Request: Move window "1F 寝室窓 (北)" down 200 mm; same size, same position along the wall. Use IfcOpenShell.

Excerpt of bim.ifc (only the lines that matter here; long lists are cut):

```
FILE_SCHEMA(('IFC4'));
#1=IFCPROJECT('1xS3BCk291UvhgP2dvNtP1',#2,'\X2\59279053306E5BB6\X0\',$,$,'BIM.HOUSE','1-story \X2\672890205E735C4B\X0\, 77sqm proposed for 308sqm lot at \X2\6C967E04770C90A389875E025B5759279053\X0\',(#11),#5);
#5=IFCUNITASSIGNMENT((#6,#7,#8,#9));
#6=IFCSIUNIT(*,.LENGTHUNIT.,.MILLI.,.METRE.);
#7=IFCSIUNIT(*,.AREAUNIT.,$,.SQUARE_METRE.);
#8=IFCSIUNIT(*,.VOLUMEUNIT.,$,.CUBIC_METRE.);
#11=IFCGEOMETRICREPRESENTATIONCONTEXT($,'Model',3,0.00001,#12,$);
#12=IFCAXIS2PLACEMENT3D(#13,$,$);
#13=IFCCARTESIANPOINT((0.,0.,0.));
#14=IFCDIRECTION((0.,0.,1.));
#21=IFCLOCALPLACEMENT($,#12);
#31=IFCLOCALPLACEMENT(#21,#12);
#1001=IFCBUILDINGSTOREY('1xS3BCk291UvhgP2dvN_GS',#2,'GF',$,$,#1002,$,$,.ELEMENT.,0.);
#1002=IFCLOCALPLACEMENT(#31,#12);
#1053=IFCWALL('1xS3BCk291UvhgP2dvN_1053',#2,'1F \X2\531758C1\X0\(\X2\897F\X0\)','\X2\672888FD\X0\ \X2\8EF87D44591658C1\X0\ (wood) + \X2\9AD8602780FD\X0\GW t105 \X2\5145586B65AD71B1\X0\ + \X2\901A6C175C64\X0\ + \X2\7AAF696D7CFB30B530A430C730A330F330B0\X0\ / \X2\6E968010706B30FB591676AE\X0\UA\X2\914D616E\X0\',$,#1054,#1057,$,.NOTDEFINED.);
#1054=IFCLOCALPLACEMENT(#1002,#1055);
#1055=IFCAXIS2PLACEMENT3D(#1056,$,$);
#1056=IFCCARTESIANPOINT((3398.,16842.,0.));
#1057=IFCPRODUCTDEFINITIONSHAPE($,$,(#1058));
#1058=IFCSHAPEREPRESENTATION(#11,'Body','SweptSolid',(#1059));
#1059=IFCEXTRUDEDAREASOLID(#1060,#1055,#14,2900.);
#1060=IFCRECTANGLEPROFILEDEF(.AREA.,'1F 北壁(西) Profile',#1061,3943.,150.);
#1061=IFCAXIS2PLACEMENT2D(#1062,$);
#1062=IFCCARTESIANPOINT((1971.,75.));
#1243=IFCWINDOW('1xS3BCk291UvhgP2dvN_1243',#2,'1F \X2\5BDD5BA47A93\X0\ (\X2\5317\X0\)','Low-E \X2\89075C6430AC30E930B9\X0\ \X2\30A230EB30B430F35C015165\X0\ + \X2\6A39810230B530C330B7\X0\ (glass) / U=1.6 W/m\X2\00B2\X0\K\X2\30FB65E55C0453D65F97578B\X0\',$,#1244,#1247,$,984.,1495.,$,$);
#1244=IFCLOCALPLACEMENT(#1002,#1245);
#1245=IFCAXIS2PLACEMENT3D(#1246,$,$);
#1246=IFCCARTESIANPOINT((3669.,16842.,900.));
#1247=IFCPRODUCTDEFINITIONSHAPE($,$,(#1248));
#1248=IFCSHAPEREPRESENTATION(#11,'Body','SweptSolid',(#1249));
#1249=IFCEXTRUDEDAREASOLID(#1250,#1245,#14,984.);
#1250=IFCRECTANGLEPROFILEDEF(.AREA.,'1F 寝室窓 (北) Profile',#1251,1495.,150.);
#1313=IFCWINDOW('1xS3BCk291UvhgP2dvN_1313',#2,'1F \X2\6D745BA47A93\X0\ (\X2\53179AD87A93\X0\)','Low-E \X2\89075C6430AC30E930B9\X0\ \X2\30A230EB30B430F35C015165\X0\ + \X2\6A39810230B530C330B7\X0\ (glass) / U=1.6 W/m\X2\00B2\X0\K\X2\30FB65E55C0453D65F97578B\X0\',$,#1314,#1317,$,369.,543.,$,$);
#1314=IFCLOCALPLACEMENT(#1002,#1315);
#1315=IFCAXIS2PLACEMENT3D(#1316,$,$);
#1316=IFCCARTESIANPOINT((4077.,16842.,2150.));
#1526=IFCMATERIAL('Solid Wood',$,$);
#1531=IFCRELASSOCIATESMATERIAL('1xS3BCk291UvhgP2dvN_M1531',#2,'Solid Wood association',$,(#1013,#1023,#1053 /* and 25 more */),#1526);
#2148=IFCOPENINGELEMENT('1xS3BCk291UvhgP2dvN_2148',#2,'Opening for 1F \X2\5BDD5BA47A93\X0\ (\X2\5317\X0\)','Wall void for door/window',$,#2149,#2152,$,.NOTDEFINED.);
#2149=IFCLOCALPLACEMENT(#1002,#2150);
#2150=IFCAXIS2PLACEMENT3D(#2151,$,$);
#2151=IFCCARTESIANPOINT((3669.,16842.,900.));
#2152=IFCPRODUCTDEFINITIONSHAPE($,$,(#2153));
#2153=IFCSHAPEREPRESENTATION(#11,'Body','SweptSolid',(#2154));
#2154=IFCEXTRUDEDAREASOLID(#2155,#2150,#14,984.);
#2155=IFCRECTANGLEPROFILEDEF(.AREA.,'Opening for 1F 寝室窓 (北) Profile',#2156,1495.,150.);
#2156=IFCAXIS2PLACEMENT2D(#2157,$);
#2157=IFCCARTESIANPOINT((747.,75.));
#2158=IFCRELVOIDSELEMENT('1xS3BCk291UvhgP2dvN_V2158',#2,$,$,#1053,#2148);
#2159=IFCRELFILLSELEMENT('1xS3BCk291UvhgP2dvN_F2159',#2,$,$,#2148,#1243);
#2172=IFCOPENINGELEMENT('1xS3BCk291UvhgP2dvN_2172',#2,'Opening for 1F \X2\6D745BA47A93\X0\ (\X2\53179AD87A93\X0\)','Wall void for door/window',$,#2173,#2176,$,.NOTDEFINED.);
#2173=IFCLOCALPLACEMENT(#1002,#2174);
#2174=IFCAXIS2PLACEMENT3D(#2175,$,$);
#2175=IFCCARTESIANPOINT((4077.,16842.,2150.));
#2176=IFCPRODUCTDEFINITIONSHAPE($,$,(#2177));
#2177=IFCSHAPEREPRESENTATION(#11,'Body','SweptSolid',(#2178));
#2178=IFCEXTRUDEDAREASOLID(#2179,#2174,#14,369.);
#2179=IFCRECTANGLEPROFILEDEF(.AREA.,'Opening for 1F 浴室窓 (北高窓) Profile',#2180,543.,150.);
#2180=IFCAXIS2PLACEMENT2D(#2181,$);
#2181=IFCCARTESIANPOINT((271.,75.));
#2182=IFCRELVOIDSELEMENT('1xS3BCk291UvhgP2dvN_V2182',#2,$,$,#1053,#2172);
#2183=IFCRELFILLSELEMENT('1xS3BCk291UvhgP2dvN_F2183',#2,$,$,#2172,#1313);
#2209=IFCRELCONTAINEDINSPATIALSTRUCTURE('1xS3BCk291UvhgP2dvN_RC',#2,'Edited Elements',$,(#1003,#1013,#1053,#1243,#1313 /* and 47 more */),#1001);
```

```python
import numpy as np
import ifcopenshell
import ifcopenshell.api.geometry
import ifcopenshell.util.placement
import ifcopenshell.util.unit

model = ifcopenshell.open("bim.ifc")
unit_scale = ifcopenshell.util.unit.calculate_unit_scale(model)

window = model.by_guid("1xS3BCk291UvhgP2dvN_1243")
opening = window.FillsVoids[0].RelatingOpeningElement
dz = -0.2 / unit_scale

shift = np.array([0.0, 0.0, dz])
# The window is not placed relative to its opening, so move both.
for product in (opening, window):
    matrix = ifcopenshell.util.placement.get_local_placement(product.ObjectPlacement)
    matrix[:3, 3] += shift
    ifcopenshell.api.geometry.edit_object_placement(model, product=product, matrix=matrix, is_si=False)

print(f"moved by {dz * unit_scale:+.3f} m")

model.write("bim-out.ifc")
```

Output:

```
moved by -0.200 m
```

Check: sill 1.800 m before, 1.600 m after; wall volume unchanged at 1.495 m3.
